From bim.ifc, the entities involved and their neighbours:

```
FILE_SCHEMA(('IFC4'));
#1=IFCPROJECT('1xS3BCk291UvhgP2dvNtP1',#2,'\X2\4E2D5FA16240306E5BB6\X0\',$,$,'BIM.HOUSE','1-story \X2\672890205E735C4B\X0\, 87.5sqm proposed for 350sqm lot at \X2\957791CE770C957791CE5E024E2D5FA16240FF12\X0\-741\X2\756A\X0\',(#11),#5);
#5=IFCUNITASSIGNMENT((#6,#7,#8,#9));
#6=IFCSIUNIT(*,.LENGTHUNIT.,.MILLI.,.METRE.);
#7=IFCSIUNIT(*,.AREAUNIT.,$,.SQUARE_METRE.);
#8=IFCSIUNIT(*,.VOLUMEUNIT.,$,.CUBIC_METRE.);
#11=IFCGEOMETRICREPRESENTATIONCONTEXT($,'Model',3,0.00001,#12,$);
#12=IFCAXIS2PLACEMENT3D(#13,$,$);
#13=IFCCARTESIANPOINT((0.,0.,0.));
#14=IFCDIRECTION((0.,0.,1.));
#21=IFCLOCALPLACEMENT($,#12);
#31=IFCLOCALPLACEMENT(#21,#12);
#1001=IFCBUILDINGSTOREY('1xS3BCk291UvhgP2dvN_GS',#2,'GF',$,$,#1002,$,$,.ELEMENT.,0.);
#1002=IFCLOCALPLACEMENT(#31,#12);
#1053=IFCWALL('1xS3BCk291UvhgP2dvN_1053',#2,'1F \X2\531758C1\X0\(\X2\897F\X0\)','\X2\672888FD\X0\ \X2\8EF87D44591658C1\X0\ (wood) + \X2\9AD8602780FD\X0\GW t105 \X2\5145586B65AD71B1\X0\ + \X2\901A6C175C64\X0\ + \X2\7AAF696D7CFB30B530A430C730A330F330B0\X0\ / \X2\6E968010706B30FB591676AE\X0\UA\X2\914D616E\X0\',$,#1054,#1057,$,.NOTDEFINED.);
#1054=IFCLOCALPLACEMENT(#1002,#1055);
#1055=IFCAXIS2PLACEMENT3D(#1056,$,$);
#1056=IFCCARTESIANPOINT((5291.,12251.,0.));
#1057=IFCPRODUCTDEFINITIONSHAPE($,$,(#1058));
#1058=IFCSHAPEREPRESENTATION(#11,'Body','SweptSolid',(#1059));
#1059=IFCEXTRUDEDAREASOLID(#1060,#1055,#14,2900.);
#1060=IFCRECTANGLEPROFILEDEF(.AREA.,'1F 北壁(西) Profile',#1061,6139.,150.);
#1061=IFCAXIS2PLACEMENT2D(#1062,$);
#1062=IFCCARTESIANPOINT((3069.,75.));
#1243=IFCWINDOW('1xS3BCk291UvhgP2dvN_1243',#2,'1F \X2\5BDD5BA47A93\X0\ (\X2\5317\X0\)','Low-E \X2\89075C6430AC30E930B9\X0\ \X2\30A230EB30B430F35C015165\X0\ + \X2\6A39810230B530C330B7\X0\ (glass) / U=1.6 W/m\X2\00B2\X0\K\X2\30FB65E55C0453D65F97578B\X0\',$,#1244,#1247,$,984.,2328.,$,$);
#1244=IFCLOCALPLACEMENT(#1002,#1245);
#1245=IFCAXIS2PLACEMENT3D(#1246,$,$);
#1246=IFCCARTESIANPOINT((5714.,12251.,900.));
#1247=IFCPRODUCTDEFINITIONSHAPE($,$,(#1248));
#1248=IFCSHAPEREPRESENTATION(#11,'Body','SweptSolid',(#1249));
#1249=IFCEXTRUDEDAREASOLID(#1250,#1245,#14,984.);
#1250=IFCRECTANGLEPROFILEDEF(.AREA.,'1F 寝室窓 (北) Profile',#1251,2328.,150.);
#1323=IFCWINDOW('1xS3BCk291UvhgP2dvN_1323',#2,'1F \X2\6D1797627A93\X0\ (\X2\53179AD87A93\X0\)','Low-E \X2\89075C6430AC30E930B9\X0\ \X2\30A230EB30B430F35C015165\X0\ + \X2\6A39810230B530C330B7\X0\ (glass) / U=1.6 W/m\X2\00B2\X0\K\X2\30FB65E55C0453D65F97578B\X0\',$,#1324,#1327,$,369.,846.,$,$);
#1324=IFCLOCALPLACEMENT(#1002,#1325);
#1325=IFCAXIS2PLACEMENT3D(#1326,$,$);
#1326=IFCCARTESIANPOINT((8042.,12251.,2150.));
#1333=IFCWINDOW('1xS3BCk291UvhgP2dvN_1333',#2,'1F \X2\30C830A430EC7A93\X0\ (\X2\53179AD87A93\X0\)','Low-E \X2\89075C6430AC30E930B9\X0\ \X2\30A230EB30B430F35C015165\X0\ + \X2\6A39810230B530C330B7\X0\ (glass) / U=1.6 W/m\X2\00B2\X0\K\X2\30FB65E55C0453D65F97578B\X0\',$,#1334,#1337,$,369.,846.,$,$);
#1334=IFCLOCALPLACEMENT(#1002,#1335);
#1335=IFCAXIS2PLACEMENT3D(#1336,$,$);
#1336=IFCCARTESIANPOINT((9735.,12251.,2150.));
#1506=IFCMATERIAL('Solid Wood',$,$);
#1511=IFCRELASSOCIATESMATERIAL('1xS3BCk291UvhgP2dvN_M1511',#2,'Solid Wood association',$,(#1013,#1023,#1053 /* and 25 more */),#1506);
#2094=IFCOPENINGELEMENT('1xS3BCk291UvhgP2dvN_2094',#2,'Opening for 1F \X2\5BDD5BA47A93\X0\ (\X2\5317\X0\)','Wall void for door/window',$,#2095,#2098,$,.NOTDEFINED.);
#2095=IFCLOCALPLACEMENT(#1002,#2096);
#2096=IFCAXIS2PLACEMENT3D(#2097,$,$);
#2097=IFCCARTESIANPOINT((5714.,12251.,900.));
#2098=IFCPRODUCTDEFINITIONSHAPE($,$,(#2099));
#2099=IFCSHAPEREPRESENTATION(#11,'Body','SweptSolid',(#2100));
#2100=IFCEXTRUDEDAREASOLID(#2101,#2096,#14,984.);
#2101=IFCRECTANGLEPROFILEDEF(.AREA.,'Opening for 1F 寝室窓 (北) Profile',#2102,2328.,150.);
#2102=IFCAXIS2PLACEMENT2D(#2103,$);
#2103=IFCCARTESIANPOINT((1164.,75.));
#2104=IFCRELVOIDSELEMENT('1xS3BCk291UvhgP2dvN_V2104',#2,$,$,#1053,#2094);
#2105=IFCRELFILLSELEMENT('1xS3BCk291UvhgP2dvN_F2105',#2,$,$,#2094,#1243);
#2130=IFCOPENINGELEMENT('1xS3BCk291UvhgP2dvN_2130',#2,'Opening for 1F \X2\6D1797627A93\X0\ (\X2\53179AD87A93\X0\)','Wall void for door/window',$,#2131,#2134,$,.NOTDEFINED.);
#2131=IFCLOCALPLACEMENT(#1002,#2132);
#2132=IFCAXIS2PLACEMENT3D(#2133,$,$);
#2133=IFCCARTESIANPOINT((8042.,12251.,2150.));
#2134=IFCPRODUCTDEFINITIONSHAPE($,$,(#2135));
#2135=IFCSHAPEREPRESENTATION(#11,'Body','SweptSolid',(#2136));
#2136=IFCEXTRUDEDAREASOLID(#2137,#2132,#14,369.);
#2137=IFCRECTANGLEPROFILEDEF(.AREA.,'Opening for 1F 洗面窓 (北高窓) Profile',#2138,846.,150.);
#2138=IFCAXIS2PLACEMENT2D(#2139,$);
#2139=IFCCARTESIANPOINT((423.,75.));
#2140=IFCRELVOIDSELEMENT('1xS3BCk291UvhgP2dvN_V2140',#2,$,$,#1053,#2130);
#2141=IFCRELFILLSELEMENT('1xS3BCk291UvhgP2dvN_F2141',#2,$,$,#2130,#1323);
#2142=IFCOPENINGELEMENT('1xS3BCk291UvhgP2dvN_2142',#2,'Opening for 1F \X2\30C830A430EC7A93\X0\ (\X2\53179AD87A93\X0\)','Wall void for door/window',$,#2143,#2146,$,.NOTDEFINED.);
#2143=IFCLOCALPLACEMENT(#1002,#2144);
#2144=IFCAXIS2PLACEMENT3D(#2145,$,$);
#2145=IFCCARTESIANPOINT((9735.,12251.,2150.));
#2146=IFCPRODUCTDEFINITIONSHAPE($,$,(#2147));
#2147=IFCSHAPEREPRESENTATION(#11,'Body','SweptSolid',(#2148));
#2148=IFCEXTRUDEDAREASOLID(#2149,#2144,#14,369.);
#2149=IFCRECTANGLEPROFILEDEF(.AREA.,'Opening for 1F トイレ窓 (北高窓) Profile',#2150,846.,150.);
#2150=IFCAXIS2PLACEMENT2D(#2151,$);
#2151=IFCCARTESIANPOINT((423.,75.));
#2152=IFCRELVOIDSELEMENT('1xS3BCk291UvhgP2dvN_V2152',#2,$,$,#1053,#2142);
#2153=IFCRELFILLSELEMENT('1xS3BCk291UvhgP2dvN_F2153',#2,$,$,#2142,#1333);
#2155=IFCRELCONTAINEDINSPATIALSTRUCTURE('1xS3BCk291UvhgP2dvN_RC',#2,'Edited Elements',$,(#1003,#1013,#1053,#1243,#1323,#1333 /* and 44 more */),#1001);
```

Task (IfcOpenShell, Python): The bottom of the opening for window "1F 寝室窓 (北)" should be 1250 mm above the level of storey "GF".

```python
import numpy as np
import ifcopenshell
import ifcopenshell.api.geometry
import ifcopenshell.geom
import ifcopenshell.util.element
import ifcopenshell.util.placement
import ifcopenshell.util.shape
import ifcopenshell.util.unit

model = ifcopenshell.open("bim.ifc")
unit_scale = ifcopenshell.util.unit.calculate_unit_scale(model)

window = model.by_id(1243)
opening = window.FillsVoids[0].RelatingOpeningElement
storey = ifcopenshell.util.element.get_container(window, ifc_class="IfcBuildingStorey")
level = ifcopenshell.util.placement.get_local_placement(storey.ObjectPlacement)[2, 3]

# The opening's origin need not be at the sill, so measure its lowest point.
shape = ifcopenshell.geom.create_shape(ifcopenshell.geom.settings(), opening)
bottom = ifcopenshell.util.shape.get_shape_bottom_elevation(shape, shape.geometry) / unit_scale
dz = level + 1.25 / unit_scale - bottom

shift = np.array([0.0, 0.0, dz])
# The window is not placed relative to its opening, so move both.
for product in (opening, window):
    matrix = ifcopenshell.util.placement.get_local_placement(product.ObjectPlacement)
    matrix[:3, 3] += shift
    ifcopenshell.api.geometry.edit_object_placement(model, product=product, matrix=matrix, is_si=False)

print(f"moved by {dz * unit_scale:+.3f} m")

model.write("bim-out.ifc")
```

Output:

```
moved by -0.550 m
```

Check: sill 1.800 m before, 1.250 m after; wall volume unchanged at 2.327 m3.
